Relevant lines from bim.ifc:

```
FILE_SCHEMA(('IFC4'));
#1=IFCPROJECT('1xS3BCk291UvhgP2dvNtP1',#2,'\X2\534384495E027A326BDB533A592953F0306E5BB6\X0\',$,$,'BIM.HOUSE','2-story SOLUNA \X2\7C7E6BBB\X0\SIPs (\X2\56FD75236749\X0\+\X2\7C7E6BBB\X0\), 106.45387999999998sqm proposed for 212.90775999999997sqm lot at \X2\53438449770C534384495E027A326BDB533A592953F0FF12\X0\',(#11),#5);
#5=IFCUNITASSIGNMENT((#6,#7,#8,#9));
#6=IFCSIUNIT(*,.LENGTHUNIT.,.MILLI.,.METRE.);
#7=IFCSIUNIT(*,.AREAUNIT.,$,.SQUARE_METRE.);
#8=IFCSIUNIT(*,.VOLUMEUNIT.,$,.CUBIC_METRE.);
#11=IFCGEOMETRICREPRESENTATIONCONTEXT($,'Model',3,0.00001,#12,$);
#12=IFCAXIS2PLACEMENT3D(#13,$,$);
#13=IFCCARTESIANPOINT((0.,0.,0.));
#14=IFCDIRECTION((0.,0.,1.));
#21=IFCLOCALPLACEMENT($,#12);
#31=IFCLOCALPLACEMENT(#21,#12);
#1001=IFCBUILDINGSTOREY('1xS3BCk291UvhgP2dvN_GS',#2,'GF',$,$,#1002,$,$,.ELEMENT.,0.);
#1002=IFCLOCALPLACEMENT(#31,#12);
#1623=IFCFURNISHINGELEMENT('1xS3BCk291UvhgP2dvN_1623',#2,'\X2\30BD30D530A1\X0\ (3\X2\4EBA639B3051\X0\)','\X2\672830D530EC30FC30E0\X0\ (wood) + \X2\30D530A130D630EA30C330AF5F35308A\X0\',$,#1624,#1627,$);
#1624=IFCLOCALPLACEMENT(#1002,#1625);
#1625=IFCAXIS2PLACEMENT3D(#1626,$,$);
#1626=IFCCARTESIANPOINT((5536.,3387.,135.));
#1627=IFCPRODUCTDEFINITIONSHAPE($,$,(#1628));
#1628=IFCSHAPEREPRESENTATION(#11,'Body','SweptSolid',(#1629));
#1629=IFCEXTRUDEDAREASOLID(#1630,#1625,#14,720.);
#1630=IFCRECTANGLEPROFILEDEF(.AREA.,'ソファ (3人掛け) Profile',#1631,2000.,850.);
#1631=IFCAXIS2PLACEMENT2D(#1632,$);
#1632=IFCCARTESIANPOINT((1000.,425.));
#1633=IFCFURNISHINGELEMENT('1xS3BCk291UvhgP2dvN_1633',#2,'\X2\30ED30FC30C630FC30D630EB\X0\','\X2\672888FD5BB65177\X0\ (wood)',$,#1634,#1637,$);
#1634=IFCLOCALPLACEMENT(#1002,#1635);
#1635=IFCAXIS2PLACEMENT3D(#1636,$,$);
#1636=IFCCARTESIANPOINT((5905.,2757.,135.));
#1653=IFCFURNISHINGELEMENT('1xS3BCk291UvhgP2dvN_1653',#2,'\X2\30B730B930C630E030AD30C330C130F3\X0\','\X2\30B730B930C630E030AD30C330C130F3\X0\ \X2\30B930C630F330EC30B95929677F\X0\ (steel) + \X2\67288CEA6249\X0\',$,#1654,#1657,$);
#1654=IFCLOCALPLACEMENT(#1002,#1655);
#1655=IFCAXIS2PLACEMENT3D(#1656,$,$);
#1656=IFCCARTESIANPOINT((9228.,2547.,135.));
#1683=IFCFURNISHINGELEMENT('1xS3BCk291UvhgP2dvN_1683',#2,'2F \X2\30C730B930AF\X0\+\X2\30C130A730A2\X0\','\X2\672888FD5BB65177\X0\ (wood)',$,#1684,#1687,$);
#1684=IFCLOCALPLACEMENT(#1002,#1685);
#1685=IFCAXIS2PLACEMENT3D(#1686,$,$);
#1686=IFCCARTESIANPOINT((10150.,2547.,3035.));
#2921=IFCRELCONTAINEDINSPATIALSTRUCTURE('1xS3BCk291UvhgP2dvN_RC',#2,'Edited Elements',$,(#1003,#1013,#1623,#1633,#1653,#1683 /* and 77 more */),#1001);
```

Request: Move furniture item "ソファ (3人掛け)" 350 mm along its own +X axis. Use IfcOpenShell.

```python
import ifcopenshell
import ifcopenshell.api.geometry
import ifcopenshell.util.placement
import ifcopenshell.util.unit

model = ifcopenshell.open("bim.ifc")
unit_scale = ifcopenshell.util.unit.calculate_unit_scale(model)

item = model.by_guid("1xS3BCk291UvhgP2dvN_1623")
matrix = ifcopenshell.util.placement.get_local_placement(item.ObjectPlacement)
matrix[:3, 3] += matrix[:3, 0] * 0.35 / unit_scale
ifcopenshell.api.geometry.edit_object_placement(model, product=item, matrix=matrix, is_si=False)

print(ifcopenshell.util.placement.get_local_placement(item.ObjectPlacement).round(3) + 0.0)

model.write("bim-out.ifc")
```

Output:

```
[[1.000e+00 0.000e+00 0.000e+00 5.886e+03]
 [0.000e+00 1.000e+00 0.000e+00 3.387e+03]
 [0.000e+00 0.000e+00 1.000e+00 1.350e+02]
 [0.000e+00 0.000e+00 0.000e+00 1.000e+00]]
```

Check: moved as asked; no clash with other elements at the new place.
